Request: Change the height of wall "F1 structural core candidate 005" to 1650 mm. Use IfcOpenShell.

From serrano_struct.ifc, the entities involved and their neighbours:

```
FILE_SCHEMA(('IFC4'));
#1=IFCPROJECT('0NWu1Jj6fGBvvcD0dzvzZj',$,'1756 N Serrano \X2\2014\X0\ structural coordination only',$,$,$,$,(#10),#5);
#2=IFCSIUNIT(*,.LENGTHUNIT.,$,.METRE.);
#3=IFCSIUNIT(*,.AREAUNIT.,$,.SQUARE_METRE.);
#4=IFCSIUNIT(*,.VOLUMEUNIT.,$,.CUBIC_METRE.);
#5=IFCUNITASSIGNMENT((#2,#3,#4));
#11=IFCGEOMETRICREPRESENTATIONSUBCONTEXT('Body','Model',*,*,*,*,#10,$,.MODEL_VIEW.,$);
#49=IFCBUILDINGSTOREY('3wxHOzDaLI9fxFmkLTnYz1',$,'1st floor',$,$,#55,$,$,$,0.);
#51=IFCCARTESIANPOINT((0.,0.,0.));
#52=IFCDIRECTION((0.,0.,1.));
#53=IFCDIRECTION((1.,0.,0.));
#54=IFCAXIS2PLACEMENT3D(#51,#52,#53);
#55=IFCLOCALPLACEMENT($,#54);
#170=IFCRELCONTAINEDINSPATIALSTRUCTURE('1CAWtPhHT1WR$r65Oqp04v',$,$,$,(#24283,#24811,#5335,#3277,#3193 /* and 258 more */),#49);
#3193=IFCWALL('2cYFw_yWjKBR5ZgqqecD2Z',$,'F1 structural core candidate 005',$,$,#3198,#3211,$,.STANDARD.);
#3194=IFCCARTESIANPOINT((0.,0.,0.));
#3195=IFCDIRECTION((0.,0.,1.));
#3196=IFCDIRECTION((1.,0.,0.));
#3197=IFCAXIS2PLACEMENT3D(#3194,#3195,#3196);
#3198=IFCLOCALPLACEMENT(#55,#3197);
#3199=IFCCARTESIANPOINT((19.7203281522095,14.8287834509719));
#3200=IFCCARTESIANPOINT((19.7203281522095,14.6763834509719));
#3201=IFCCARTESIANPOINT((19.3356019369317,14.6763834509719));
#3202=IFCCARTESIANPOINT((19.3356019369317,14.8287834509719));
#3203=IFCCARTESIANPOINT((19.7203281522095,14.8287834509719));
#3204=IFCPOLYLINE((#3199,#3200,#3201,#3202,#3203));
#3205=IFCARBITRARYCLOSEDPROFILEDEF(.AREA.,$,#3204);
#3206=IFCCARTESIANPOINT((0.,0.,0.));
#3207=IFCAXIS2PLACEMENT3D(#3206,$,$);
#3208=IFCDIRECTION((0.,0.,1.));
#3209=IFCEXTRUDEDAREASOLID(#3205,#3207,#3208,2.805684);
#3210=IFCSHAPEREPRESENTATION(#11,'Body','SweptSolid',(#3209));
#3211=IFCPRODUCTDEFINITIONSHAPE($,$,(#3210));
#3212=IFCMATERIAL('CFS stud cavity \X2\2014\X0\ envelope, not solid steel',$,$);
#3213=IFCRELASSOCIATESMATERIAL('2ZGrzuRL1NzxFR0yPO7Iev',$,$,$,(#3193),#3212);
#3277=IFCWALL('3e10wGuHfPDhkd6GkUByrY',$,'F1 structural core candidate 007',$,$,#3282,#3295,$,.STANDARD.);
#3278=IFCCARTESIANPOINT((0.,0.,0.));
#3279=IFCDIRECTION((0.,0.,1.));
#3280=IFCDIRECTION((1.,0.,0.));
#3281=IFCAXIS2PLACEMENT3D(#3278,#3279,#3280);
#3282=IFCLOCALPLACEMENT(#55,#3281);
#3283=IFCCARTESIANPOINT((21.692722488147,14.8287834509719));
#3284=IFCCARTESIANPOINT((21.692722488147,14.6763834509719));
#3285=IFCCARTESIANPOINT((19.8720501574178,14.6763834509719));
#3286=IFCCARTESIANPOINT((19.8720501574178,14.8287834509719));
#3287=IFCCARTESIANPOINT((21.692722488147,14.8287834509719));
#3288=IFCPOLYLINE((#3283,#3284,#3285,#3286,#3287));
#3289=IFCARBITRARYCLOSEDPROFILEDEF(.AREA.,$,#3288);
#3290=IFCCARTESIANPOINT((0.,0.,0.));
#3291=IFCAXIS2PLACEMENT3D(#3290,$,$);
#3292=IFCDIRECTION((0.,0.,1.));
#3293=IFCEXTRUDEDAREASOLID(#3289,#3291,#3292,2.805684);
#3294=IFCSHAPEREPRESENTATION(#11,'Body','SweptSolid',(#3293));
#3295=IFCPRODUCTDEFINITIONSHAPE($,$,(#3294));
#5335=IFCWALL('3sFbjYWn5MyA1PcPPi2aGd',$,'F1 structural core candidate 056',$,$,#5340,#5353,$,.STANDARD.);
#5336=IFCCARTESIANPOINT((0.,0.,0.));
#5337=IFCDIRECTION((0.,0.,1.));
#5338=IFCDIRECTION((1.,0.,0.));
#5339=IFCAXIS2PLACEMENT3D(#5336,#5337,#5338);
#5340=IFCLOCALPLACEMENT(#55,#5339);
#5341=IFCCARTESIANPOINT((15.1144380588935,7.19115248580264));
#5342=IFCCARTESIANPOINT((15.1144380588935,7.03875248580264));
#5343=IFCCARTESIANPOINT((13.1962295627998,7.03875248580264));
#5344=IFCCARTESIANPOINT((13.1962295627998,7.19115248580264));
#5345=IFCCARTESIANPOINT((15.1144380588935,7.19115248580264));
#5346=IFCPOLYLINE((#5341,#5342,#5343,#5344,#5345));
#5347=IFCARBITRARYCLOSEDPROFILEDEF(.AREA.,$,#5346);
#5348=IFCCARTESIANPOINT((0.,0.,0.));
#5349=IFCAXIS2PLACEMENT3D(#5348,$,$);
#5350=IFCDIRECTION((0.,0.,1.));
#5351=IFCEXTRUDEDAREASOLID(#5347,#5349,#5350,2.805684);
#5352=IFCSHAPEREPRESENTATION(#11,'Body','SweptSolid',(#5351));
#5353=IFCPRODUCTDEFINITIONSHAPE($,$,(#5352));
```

```python
import ifcopenshell
import ifcopenshell.geom
import ifcopenshell.util.representation
import ifcopenshell.util.shape
import ifcopenshell.util.unit

model = ifcopenshell.open("serrano_struct.ifc")
unit_scale = ifcopenshell.util.unit.calculate_unit_scale(model)
settings = ifcopenshell.geom.settings()


def volume(element):
    """Net volume in cubic metres, openings subtracted."""
    shape = ifcopenshell.geom.create_shape(settings, element)
    return ifcopenshell.util.shape.get_volume(shape.geometry)


wall = model.by_id(3193)
before = volume(wall)

body = ifcopenshell.util.representation.get_representation(wall, "Model", "Body")
solid = body.Items[0]
old_height = solid.Depth
solid.Depth = 1.65 / unit_scale
after = volume(wall)

print(f"height {old_height:g} -> {solid.Depth:g}, volume {before:.3f} -> {after:.3f} m3")

model.write("serrano_struct_edited.ifc")
```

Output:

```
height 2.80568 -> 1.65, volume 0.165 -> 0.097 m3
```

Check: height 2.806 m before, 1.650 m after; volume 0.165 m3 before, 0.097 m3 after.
